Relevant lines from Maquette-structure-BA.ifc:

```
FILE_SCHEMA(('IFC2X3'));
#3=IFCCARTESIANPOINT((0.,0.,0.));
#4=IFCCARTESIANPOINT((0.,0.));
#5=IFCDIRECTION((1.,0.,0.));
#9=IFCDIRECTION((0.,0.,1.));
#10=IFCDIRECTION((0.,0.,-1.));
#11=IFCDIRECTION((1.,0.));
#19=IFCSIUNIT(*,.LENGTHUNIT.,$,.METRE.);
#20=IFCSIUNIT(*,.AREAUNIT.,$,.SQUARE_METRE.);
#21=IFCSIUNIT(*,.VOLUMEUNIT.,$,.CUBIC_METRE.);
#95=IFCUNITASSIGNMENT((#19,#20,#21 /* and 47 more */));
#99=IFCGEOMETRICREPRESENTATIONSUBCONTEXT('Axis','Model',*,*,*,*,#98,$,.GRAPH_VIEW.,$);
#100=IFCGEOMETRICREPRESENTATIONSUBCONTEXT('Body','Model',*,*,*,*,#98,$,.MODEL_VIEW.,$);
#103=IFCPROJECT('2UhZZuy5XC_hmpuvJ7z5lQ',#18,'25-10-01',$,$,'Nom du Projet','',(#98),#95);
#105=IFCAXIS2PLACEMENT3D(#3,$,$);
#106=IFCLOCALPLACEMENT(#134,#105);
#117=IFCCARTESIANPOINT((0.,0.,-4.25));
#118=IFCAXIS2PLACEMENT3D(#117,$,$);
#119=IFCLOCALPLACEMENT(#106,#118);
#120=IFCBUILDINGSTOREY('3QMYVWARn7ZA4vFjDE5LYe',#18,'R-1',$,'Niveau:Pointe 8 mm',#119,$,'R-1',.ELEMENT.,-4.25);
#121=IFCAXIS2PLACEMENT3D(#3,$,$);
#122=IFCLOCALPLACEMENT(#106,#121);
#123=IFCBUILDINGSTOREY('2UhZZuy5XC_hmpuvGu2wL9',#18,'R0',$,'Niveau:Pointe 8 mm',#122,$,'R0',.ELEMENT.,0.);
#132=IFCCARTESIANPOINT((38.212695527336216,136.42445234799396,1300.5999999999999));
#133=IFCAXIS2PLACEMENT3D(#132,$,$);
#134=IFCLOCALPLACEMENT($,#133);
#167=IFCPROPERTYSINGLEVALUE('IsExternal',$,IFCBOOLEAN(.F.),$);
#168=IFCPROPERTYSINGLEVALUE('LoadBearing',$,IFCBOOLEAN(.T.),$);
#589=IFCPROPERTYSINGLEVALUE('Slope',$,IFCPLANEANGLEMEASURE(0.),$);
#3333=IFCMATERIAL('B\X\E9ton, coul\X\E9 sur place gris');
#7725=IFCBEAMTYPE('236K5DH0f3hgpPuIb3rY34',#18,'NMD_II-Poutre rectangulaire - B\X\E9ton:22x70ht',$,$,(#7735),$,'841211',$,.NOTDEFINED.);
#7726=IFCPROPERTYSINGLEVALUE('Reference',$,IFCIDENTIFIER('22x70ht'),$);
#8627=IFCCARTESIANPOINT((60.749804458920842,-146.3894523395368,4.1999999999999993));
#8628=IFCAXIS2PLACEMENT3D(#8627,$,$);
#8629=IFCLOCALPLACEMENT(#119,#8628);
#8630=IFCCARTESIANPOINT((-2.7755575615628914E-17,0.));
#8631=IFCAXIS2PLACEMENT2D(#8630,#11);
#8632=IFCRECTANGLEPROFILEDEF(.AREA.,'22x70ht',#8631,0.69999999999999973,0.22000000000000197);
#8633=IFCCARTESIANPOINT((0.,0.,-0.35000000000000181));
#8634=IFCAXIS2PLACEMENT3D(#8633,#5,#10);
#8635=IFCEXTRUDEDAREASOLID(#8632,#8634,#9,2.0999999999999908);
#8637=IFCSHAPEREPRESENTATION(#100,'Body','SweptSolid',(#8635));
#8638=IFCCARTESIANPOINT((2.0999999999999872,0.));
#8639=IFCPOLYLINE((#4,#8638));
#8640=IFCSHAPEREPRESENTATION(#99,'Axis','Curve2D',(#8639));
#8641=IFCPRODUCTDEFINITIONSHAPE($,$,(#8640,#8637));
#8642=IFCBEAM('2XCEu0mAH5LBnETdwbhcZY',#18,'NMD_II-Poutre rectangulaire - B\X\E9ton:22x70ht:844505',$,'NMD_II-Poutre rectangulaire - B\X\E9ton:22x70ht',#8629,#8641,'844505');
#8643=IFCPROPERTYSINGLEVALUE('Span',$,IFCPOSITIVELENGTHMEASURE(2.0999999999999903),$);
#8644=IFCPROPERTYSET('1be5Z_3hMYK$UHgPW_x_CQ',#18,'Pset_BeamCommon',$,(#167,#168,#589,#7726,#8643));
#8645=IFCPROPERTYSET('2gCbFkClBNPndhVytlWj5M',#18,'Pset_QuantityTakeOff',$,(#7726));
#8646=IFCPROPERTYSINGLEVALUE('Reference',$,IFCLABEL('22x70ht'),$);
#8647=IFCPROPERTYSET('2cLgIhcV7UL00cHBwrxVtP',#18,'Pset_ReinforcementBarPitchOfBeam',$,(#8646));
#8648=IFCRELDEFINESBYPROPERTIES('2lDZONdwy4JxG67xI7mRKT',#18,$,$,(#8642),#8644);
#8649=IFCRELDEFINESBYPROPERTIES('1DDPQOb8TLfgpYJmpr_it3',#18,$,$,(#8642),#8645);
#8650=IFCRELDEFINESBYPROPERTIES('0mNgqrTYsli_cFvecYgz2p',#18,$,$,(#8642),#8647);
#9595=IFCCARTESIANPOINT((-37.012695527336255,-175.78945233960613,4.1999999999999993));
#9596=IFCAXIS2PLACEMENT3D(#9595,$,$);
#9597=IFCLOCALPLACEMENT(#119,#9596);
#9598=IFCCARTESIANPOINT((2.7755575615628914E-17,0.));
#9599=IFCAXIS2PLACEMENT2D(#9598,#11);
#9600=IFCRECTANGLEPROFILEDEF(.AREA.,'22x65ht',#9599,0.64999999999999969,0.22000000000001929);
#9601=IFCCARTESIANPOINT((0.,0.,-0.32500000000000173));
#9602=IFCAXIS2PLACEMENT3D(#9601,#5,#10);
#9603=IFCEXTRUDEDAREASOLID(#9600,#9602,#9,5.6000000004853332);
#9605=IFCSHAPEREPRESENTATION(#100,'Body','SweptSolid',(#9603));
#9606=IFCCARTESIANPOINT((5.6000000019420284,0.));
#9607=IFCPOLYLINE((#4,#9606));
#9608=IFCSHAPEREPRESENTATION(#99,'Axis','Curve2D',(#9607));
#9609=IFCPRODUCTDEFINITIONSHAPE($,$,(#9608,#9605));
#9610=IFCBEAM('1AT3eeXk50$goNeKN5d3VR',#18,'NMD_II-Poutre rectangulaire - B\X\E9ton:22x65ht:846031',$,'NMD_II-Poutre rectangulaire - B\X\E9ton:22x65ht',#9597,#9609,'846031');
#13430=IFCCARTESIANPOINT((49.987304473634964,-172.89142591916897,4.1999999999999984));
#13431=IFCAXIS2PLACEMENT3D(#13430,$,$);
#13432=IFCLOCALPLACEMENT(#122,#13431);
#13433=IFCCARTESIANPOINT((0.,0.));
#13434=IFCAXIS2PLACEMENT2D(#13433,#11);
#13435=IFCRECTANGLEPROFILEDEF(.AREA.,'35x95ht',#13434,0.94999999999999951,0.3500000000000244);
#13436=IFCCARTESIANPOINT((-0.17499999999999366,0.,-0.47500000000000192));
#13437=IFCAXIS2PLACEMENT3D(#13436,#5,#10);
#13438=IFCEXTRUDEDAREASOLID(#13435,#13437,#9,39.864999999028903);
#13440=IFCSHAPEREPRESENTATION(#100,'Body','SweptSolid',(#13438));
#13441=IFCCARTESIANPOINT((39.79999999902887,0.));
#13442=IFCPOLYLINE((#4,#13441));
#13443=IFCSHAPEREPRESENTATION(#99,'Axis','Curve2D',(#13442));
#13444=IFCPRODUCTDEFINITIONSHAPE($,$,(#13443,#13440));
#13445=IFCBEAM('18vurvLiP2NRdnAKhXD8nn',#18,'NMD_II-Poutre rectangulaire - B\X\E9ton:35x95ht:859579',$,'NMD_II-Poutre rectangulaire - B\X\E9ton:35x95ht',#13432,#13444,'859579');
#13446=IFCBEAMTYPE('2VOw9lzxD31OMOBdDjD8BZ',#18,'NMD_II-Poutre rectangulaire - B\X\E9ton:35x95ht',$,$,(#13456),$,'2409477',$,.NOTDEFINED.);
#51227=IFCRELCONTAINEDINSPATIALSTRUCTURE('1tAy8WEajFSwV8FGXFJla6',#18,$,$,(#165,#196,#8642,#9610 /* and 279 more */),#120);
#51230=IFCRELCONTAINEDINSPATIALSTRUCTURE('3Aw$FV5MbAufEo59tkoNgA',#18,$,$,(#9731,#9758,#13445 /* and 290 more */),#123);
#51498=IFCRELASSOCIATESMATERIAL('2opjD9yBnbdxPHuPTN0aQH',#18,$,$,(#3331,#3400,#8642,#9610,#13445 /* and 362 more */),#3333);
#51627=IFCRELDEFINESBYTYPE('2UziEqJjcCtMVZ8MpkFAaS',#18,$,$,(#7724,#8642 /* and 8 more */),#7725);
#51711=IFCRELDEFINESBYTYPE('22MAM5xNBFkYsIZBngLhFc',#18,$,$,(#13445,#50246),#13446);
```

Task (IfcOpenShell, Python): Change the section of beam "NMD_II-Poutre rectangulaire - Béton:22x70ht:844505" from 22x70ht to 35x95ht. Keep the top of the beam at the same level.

```python
import ifcopenshell
import ifcopenshell.api.pset
import ifcopenshell.api.type
import ifcopenshell.util.element
import ifcopenshell.util.representation

model = ifcopenshell.open("Maquette-structure-BA.ifc")

member = model.by_guid("2XCEu0mAH5LBnETdwbhcZY")
source = next(p for p in model.by_type("IfcRectangleProfileDef") if p.ProfileName == "35x95ht")

body = ifcopenshell.util.representation.get_representation(member, "Model", "Body")
solid = body.Items[0]
old_profile = solid.SweptArea

# Copy the section's sizes but keep this member's own profile position.
profile = ifcopenshell.util.element.copy(model, source)
# Profiles are centred, so shift by half the change in depth to hold the top.
shift = (old_profile.XDim - profile.XDim) / 2
x, y = old_profile.Position.Location.Coordinates
up = (-1.0, 0.0)  # upwards, in the solid's own plane
location = model.createIfcCartesianPoint((x + up[0] * shift, y + up[1] * shift))
profile.Position = model.createIfcAxis2Placement2D(location, old_profile.Position.RefDirection)
solid.SweptArea = profile
if not model.get_total_inverses(old_profile):
    ifcopenshell.util.element.remove_deep2(model, old_profile)

new_type = model.by_guid("2VOw9lzxD31OMOBdDjD8BZ")
ifcopenshell.api.type.assign_type(
    model, related_objects=[member], relating_type=new_type, should_map_representations=False
)
member.Name = member.Name.replace("22x70ht", "35x95ht")
member.ObjectType = "NMD_II-Poutre rectangulaire - Béton:35x95ht"
pset = model.by_id(ifcopenshell.util.element.get_pset(member, "Pset_BeamCommon", should_inherit=False)["id"])
ifcopenshell.api.pset.edit_pset(model, pset=pset, properties={"Reference": "35x95ht"})
pset = model.by_id(ifcopenshell.util.element.get_pset(member, "Pset_QuantityTakeOff", should_inherit=False)["id"])
ifcopenshell.api.pset.edit_pset(model, pset=pset, properties={"Reference": "35x95ht"})
pset = model.by_id(ifcopenshell.util.element.get_pset(member, "Pset_ReinforcementBarPitchOfBeam", should_inherit=False)["id"])
ifcopenshell.api.pset.edit_pset(model, pset=pset, properties={"Reference": "35x95ht"})

print(solid.SweptArea)

model.write("Maquette-structure-BA_v2.ifc")
```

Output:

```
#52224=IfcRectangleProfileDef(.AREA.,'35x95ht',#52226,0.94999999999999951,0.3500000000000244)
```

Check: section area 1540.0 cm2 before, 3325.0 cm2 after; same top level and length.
